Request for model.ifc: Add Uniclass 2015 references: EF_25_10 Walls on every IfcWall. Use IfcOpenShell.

First a look at what the model holds.

```python
import ifcopenshell

model = ifcopenshell.open("model.ifc")
print(model.schema)
print("classifications:", [c.Name for c in model.by_type("IfcClassification")])
for ifc_class in ("IfcDoor", "IfcRoof", "IfcStair", "IfcWall", "IfcWindow"):
    print(ifc_class, len(model.by_type(ifc_class)))
```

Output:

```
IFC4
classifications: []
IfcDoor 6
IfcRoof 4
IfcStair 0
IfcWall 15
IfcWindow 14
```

```python
import ifcopenshell
import ifcopenshell.api.classification

model = ifcopenshell.open("model.ifc")

system = ifcopenshell.api.classification.add_classification(model, classification="Uniclass 2015")

codes = {
    "IfcWall": ("EF_25_10", "Walls"),
}
for ifc_class, (code, name) in codes.items():
    products = model.by_type(ifc_class)
    ifcopenshell.api.classification.add_reference(
        model, products=products, classification=system, identification=code, name=name
    )
    print(code, len(products))

model.write("model_v2.ifc")
```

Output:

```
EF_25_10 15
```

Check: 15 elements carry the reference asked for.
